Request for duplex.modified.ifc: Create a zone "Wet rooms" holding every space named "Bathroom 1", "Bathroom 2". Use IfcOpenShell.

First a look at what the model holds.

```python
import ifcopenshell

model = ifcopenshell.open("duplex.modified.ifc")
print(model.schema)
seen = {}
for space in model.by_type("IfcSpace"):
    seen[space.LongName] = seen.get(space.LongName, 0) + 1
for name, count in sorted(seen.items(), key=str):
    print(count, "x", name)
print("zones:", [z.Name for z in model.by_type("IfcZone")][:20])
```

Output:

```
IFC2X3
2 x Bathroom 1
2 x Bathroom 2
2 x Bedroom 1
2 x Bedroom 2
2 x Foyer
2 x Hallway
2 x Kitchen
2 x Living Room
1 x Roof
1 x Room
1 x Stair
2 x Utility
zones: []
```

```python
import ifcopenshell
import ifcopenshell.api.group
import ifcopenshell.api.root

model = ifcopenshell.open("duplex.modified.ifc")

names = {"Bathroom 1", "Bathroom 2"}
spaces = [s for s in model.by_type("IfcSpace") if s.LongName in names]

zone = ifcopenshell.api.root.create_entity(model, ifc_class="IfcZone", name="Wet rooms")
ifcopenshell.api.group.assign_group(model, products=spaces, group=zone)
print(len(spaces), "spaces in", zone.Name)

model.write("duplex.modified_v2.ifc")
```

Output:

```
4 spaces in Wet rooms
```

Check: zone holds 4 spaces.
